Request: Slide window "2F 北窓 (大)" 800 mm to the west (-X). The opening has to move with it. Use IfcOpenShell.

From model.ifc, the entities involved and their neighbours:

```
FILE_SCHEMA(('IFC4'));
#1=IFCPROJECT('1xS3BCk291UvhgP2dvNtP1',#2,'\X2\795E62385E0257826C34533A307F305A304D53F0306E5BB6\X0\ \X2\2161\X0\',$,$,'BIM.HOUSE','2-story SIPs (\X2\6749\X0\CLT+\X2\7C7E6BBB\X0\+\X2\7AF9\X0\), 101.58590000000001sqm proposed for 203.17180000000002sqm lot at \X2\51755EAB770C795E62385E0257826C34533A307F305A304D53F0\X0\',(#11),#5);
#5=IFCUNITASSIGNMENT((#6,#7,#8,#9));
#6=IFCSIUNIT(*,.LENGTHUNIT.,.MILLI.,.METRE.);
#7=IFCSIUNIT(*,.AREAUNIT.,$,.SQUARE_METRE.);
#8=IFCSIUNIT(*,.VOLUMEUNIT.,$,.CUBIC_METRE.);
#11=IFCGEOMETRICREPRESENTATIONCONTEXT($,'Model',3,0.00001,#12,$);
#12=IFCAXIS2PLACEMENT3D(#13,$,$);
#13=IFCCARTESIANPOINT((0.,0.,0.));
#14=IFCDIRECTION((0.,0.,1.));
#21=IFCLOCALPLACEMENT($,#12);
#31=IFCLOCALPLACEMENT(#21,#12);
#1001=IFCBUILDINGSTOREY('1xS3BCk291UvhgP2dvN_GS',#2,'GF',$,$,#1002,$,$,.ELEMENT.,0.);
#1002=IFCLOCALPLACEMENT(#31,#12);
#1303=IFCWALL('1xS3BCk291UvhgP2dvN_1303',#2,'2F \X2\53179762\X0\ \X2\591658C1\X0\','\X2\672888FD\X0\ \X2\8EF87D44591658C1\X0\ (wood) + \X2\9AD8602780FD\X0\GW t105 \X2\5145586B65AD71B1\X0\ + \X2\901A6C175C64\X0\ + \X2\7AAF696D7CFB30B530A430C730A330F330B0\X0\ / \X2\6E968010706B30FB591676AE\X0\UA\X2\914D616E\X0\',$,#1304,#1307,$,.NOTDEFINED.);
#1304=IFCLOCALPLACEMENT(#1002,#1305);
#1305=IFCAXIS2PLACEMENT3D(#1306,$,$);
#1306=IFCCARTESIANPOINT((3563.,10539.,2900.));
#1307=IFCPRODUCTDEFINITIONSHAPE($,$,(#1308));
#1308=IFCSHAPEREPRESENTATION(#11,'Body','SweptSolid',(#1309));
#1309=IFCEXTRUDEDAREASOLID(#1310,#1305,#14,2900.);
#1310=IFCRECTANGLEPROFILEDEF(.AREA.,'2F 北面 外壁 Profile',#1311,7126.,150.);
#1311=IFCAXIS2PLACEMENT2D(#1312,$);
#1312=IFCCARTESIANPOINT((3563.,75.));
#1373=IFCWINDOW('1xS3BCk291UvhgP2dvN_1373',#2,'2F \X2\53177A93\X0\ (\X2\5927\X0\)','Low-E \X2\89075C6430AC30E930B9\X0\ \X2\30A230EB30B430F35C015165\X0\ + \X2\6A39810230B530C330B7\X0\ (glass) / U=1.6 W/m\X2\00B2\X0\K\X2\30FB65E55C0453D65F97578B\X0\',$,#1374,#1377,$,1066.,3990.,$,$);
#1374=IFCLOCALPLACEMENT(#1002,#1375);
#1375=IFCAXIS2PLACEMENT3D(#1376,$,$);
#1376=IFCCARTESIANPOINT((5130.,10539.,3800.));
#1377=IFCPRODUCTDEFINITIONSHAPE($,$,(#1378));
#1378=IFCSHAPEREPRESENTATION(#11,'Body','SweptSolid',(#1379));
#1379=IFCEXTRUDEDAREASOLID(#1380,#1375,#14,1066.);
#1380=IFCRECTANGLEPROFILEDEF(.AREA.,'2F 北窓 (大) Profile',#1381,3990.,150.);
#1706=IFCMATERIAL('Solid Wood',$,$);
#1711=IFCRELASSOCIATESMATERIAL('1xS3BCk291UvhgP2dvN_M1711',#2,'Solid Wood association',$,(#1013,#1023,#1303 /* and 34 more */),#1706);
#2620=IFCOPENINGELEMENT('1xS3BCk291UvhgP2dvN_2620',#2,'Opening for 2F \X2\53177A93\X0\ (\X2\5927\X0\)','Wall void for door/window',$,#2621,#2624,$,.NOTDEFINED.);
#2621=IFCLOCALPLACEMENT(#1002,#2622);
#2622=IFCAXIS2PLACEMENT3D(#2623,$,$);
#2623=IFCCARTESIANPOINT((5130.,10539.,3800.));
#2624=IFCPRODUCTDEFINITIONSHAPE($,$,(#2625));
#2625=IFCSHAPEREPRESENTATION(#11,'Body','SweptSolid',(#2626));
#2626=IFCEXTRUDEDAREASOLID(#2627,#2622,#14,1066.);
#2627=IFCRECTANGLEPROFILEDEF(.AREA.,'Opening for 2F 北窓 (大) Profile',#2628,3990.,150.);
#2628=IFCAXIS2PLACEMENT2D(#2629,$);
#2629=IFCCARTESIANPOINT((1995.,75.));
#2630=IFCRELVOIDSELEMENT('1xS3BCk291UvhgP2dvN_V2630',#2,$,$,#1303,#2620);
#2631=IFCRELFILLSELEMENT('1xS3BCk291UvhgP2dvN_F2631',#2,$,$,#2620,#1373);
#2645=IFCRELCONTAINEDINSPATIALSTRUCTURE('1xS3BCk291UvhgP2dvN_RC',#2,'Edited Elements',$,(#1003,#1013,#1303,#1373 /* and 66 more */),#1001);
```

```python
import ifcopenshell
import ifcopenshell.api.geometry
import ifcopenshell.util.placement
import ifcopenshell.util.unit

model = ifcopenshell.open("model.ifc")
unit_scale = ifcopenshell.util.unit.calculate_unit_scale(model)

window = model.by_guid("1xS3BCk291UvhgP2dvN_1373")
opening = window.FillsVoids[0].RelatingOpeningElement
wall = opening.VoidsElements[0].RelatingBuildingElement

wall_matrix = ifcopenshell.util.placement.get_local_placement(wall.ObjectPlacement)
shift = wall_matrix[:3, 0] * -0.8 / unit_scale
before = ifcopenshell.util.placement.get_local_placement(window.ObjectPlacement)[:3, 3].copy()

# The window is not placed relative to its opening, so move both.
for product in (opening, window):
    matrix = ifcopenshell.util.placement.get_local_placement(product.ObjectPlacement)
    matrix[:3, 3] += shift
    ifcopenshell.api.geometry.edit_object_placement(model, product=product, matrix=matrix, is_si=False)

after = ifcopenshell.util.placement.get_local_placement(window.ObjectPlacement)[:3, 3]
print("window moved by", (after - before).round(3) + 0.0)

model.write("model_v2.ifc")
```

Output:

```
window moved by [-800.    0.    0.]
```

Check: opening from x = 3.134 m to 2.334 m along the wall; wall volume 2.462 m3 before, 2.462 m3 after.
